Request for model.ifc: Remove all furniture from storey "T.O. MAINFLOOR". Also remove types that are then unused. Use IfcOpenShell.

First a look at what the model holds.

```python
import ifcopenshell
import ifcopenshell.util.element

model = ifcopenshell.open("model.ifc")
print(model.schema)
storey = next(s for s in model.by_type("IfcBuildingStorey") if s.Name == "T.O. MAINFLOOR")
furniture = [e for e in ifcopenshell.util.element.get_decomposition(storey) if e.is_a("IfcFurnishingElement")]
seen = {}
for e in furniture:
    element_type = ifcopenshell.util.element.get_type(e)
    name = element_type.Name if element_type not in (None, e) else None
    seen[name] = seen.get(name, 0) + 1
for name, count in sorted(seen.items(), key=str):
    print(count, "x", name)
```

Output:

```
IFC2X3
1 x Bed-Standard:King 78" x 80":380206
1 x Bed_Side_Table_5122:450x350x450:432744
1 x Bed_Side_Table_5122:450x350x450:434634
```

```python
import ifcopenshell
import ifcopenshell.api.root
import ifcopenshell.util.element

model = ifcopenshell.open("model.ifc")

storey = next(s for s in model.by_type("IfcBuildingStorey") if s.Name == "T.O. MAINFLOOR")
furniture = [e for e in ifcopenshell.util.element.get_decomposition(storey) if e.is_a("IfcFurnishingElement")]
types = {ifcopenshell.util.element.get_type(e) for e in furniture} - {None, *furniture}

for e in furniture:
    ifcopenshell.api.root.remove_product(model, product=e)
print(len(furniture), "removed")

unused = [t for t in types if not ifcopenshell.util.element.get_types(t)]
for t in unused:
    ifcopenshell.api.root.remove_product(model, product=t)
print(len(unused), "unused types removed")

model.write("model_updated.ifc")
```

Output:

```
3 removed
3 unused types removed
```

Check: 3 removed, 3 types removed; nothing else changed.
